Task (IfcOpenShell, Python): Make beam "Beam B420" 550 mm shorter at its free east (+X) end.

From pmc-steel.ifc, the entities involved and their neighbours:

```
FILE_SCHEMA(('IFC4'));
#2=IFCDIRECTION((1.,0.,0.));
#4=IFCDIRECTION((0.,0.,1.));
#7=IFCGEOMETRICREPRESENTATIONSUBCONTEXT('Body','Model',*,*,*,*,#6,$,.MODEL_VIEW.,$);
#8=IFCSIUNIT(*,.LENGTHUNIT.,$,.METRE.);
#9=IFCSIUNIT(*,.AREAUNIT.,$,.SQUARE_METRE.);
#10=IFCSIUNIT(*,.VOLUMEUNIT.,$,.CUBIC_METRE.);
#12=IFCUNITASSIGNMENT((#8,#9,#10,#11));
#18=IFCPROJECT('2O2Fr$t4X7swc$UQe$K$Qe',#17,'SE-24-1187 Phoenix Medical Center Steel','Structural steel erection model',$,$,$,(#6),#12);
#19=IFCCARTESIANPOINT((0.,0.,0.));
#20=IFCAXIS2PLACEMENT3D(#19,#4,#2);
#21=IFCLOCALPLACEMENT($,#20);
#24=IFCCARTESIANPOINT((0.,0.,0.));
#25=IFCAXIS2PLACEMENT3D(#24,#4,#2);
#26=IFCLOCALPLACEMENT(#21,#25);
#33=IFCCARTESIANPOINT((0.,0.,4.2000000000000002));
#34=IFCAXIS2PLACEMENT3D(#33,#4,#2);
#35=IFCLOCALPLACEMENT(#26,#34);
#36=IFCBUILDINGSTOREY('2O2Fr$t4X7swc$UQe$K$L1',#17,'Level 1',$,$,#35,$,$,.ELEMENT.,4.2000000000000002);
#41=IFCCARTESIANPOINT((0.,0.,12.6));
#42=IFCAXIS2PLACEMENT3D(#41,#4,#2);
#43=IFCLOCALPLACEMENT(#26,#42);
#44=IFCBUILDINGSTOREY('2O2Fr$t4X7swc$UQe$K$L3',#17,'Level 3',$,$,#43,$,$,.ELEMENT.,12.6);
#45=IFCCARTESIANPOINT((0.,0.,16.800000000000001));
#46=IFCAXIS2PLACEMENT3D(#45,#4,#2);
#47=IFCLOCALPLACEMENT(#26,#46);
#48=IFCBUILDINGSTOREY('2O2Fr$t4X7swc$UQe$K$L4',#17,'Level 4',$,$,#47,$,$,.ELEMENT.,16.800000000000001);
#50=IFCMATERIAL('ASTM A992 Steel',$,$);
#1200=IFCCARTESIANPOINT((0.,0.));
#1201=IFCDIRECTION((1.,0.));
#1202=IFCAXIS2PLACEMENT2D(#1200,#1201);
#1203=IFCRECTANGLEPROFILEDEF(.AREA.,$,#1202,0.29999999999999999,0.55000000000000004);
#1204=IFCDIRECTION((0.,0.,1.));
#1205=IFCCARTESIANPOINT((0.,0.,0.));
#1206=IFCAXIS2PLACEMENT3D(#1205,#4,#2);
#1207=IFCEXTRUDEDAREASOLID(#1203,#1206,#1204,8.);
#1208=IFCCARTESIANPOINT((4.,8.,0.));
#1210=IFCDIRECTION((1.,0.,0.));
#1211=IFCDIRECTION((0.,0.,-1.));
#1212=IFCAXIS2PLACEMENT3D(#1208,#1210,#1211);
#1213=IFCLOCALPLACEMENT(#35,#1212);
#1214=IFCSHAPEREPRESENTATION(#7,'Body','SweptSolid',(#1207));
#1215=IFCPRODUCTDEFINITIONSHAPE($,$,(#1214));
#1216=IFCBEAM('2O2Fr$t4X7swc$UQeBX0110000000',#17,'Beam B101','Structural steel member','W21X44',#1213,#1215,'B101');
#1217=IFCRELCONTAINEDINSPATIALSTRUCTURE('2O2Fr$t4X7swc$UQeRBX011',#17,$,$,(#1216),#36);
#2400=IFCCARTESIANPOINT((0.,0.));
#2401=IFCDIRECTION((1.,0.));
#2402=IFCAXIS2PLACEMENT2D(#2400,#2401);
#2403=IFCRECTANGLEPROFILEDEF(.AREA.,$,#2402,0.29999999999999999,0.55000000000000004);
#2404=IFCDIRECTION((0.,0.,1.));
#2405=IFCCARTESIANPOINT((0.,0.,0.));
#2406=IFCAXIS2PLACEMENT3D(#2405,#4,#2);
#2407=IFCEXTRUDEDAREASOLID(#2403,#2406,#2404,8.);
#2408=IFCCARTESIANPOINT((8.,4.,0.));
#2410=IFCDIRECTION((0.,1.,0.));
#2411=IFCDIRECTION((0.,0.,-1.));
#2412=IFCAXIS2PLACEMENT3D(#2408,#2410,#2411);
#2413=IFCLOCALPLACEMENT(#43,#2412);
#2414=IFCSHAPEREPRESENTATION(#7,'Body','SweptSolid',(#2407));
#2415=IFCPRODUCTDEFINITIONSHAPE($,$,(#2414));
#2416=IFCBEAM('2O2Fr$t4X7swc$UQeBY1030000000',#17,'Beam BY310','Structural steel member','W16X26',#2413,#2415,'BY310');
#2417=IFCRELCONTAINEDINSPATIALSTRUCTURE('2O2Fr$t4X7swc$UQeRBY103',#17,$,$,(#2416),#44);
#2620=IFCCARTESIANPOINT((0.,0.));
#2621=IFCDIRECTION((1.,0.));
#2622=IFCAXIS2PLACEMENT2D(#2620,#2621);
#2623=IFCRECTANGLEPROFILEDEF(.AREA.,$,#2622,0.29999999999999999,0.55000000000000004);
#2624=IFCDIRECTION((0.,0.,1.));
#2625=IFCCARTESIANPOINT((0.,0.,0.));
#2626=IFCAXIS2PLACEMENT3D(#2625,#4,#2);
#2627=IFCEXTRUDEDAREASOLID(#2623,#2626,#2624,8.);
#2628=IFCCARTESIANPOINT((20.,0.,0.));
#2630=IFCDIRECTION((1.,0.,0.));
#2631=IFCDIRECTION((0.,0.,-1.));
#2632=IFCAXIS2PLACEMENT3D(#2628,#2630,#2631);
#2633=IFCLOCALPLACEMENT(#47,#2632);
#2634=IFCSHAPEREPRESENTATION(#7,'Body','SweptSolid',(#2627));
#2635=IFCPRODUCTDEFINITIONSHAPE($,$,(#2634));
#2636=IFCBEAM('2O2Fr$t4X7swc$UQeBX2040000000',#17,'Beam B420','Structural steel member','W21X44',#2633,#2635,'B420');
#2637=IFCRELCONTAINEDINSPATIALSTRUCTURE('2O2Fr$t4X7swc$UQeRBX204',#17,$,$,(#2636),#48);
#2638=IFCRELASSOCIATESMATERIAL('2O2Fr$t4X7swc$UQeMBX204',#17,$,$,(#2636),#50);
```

```python
import ifcopenshell
import ifcopenshell.util.representation

model = ifcopenshell.open("pmc-steel.ifc")

member = model.by_guid("2O2Fr$t4X7swc$UQeBX2040000000")
change = -0.55

# The extrusion runs towards the end named, so only its depth changes.
body = ifcopenshell.util.representation.get_representation(member, "Model", "Body")
solid = body.Items[0]
old_length = solid.Depth
solid.Depth += change

print(f"length {old_length:g} -> {solid.Depth:g}")

model.write("pmc-steel_v2.ifc")
```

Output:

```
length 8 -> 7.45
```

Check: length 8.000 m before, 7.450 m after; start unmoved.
